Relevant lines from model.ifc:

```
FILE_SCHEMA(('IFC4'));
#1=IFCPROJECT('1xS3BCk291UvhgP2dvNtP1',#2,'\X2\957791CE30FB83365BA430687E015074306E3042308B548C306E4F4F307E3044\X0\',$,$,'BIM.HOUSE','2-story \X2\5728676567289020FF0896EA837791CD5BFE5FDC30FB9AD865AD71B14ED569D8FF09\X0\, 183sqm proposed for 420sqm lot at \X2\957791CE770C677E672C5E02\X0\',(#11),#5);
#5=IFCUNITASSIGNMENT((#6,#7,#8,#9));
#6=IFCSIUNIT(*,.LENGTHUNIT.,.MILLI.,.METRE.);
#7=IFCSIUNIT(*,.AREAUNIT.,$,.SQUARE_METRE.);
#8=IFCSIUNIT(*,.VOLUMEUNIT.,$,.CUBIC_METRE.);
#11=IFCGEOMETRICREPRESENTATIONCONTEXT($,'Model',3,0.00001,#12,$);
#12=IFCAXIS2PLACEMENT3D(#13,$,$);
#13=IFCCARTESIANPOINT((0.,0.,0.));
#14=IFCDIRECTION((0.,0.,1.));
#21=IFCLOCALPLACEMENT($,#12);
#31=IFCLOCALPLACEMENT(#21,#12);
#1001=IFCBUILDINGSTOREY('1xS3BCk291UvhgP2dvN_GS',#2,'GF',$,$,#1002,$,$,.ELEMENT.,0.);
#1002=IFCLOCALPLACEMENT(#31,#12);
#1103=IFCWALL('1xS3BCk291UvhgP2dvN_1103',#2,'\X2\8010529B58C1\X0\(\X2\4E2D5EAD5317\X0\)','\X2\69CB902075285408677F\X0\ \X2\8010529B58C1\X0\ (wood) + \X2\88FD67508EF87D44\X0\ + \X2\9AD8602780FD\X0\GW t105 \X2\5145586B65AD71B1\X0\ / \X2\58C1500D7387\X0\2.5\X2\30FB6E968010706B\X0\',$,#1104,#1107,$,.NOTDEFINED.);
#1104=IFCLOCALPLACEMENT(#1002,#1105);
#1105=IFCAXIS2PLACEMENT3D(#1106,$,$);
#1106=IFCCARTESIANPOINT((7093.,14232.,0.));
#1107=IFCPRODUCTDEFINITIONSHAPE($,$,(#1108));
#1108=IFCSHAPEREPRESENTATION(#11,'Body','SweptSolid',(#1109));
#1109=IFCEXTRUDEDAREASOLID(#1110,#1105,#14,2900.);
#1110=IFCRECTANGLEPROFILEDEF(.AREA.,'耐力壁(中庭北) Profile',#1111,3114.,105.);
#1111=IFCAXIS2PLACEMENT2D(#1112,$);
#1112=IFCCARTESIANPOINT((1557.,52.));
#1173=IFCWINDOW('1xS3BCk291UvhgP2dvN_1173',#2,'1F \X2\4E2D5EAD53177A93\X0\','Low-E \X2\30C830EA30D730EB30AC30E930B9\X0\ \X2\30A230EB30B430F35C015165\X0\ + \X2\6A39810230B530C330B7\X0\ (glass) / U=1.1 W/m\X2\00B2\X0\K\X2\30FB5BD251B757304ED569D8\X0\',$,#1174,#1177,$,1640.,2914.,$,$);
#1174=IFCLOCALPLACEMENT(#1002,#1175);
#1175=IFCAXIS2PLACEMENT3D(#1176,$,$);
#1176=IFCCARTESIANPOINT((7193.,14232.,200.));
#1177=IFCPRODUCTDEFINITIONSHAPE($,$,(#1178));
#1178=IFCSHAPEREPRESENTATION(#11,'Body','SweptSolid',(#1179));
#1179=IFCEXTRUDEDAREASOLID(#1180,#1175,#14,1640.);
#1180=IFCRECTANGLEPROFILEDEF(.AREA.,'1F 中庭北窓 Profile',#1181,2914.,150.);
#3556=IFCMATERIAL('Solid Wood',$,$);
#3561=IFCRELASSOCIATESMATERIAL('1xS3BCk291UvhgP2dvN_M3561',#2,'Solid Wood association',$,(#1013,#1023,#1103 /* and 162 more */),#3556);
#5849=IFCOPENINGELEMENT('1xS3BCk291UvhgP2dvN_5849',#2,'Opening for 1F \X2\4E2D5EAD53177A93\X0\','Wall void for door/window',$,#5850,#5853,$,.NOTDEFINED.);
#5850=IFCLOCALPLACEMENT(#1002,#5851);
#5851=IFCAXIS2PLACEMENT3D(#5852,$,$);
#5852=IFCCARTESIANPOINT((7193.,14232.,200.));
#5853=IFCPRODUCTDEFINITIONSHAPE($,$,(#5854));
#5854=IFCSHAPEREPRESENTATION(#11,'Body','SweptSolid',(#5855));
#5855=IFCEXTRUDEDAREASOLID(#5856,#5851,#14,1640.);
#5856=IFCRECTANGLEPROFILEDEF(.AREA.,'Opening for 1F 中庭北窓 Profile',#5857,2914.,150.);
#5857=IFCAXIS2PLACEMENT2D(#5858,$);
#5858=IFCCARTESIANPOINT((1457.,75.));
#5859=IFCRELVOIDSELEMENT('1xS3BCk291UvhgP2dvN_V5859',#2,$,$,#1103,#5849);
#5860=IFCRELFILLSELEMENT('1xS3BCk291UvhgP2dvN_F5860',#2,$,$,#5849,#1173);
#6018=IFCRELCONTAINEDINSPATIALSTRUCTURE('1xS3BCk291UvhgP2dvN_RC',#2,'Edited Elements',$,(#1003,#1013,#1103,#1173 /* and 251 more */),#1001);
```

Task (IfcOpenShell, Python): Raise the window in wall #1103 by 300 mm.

```python
import numpy as np
import ifcopenshell
import ifcopenshell.api.geometry
import ifcopenshell.util.placement
import ifcopenshell.util.unit

model = ifcopenshell.open("model.ifc")
unit_scale = ifcopenshell.util.unit.calculate_unit_scale(model)

window = model.by_guid("1xS3BCk291UvhgP2dvN_1173")
opening = window.FillsVoids[0].RelatingOpeningElement
dz = 300.0

shift = np.array([0.0, 0.0, dz])
# The window is not placed relative to its opening, so move both.
for product in (opening, window):
    matrix = ifcopenshell.util.placement.get_local_placement(product.ObjectPlacement)
    matrix[:3, 3] += shift
    ifcopenshell.api.geometry.edit_object_placement(model, product=product, matrix=matrix, is_si=False)

print(f"moved by {dz * unit_scale:+.3f} m")

model.write("model_rev.ifc")
```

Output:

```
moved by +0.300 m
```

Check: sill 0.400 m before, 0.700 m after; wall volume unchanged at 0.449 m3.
